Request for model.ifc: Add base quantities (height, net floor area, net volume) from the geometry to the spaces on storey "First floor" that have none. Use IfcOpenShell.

First a look at what the model holds.

```python
import ifcopenshell
import ifcopenshell.util.element
import ifcopenshell.util.unit

model = ifcopenshell.open("model.ifc")
print(model.schema)
for unit_type in ("LENGTHUNIT", "AREAUNIT", "VOLUMEUNIT"):
    print(unit_type, ifcopenshell.util.unit.calculate_unit_scale(model, unit_type))
storey = next(s for s in model.by_type("IfcBuildingStorey") if s.Name == "First floor")
spaces = [e for e in ifcopenshell.util.element.get_decomposition(storey) if e.is_a("IfcSpace")]
for e in sorted(spaces, key=lambda e: e.id()):
    print(e.id(), e.is_a(), e.Name, list(ifcopenshell.util.element.get_psets(e, qtos_only=True)), sep=" | ")
```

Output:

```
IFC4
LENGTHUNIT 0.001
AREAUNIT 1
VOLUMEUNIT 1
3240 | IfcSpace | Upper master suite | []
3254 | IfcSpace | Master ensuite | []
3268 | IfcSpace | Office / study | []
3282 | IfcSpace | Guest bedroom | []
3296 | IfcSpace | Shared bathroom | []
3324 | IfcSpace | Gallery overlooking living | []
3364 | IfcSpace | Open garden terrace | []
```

```python
import ifcopenshell
import ifcopenshell.api.pset
import ifcopenshell.geom
import ifcopenshell.util.element
import ifcopenshell.util.shape
import ifcopenshell.util.unit

model = ifcopenshell.open("model.ifc")
unit_scale = ifcopenshell.util.unit.calculate_unit_scale(model)
area_scale = ifcopenshell.util.unit.calculate_unit_scale(model, "AREAUNIT")
volume_scale = ifcopenshell.util.unit.calculate_unit_scale(model, "VOLUMEUNIT")
settings = ifcopenshell.geom.settings()

storey = next(s for s in model.by_type("IfcBuildingStorey") if s.Name == "First floor")
spaces = [e for e in ifcopenshell.util.element.get_decomposition(storey) if e.is_a("IfcSpace")]

for e in sorted(spaces, key=lambda e: e.id()):
    if ifcopenshell.util.element.get_psets(e, qtos_only=True, should_inherit=False):
        continue
    # Geometry comes back in metres, in the element's own axes.
    shape = ifcopenshell.geom.create_shape(settings, e)
    values = {
        "Height": ifcopenshell.util.shape.get_z(shape.geometry) / unit_scale,
        "NetFloorArea": ifcopenshell.util.shape.get_footprint_area(shape.geometry) / area_scale,
        "NetVolume": ifcopenshell.util.shape.get_volume(shape.geometry) / volume_scale,
    }
    qto = ifcopenshell.api.pset.add_qto(model, product=e, name="Qto_SpaceBaseQuantities")
    ifcopenshell.api.pset.edit_qto(model, qto=qto, properties=values)
    print(e.id(), {k: round(v, 3) for k, v in values.items()})

model.write("model_updated.ifc")
```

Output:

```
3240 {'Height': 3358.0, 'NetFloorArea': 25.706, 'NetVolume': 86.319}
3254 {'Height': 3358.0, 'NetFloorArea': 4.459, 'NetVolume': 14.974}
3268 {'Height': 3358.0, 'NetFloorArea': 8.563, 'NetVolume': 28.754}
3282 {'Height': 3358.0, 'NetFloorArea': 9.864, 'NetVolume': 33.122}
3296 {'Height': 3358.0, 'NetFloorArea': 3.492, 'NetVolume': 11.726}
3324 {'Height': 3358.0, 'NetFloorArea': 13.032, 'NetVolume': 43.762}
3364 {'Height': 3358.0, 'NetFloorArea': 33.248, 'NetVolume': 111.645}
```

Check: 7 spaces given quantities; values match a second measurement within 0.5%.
